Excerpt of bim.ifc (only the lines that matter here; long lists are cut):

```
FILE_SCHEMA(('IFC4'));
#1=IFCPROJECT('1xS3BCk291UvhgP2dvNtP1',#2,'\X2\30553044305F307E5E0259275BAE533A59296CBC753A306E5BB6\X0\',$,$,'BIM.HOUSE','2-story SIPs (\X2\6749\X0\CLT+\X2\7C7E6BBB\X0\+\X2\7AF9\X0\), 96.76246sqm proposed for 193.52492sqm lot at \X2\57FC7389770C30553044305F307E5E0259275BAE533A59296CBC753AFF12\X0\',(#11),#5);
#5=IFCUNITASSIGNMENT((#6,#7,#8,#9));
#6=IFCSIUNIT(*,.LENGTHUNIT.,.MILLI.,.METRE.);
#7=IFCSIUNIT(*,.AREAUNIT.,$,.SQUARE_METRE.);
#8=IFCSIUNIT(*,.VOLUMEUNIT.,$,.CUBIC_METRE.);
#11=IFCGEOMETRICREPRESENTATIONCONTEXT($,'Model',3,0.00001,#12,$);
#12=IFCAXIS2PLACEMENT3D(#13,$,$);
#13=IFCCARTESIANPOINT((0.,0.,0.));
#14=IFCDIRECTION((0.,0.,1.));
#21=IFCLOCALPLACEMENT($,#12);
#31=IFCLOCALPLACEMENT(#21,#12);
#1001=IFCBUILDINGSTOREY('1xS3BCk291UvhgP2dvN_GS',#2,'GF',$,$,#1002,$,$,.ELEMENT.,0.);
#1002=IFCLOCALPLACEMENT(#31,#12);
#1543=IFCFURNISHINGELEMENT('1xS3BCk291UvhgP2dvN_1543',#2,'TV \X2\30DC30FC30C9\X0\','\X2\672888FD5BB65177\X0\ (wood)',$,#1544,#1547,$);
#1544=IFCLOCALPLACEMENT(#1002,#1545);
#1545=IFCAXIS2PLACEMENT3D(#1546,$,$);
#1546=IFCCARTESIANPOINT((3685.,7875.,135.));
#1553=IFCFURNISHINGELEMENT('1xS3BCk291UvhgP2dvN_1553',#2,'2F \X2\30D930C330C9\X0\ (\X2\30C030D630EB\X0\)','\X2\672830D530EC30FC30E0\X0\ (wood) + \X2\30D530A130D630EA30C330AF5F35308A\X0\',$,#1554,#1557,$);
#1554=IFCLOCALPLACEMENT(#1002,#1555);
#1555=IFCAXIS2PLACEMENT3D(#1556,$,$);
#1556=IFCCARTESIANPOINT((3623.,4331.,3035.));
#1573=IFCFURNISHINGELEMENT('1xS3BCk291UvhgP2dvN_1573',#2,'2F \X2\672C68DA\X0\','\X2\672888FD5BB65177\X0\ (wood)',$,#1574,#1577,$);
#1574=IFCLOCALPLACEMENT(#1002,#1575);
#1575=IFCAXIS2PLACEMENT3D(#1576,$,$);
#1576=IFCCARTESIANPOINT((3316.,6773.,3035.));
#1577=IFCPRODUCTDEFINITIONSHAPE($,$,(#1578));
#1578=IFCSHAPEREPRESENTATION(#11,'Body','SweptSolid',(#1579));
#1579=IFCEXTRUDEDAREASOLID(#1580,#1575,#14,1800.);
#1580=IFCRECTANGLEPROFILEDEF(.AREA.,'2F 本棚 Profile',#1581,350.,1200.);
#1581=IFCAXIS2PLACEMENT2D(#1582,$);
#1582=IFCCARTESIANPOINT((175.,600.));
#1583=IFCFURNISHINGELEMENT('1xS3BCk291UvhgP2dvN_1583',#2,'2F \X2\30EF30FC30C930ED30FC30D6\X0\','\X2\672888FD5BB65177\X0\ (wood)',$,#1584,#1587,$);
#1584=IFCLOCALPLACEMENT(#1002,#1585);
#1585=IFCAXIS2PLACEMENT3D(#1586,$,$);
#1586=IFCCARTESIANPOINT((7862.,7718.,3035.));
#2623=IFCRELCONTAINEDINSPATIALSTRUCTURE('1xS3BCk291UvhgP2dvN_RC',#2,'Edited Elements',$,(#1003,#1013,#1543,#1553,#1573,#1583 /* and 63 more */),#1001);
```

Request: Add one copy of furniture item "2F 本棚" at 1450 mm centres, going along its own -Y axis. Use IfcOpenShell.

```python
import ifcopenshell
import ifcopenshell.api.geometry
import ifcopenshell.api.root
import ifcopenshell.util.element
import ifcopenshell.util.placement

model = ifcopenshell.open("bim.ifc")


def reuse_history(source, copy):
    """copy_class also copies each property set's owner history, people and application; keep the originals."""
    for rel in copy.IsDefinedBy:
        if rel.is_a("IfcRelDefinesByProperties") and (history := rel.RelatingPropertyDefinition.OwnerHistory):
            rel.RelatingPropertyDefinition.OwnerHistory = source.OwnerHistory
            ifcopenshell.util.element.remove_deep2(model, history)


source = model.by_guid("1xS3BCk291UvhgP2dvN_1573")
base = ifcopenshell.util.placement.get_local_placement(source.ObjectPlacement)
step = -base[:3, 1] * 1450.0

for i in range(1, 2):
    copy = ifcopenshell.api.root.copy_class(model, product=source)
    copy.Representation = ifcopenshell.util.element.copy_deep(
        model, source.Representation, exclude=["IfcGeometricRepresentationContext", "IfcRepresentationMap"]
    )
    reuse_history(source, copy)
    matrix = base.copy()
    matrix[:3, 3] += i * step
    print("added at", matrix[:3, 3].round(3) + 0.0)
    ifcopenshell.api.geometry.edit_object_placement(model, product=copy, matrix=matrix, is_si=False)

model.write("bim-out.ifc")
```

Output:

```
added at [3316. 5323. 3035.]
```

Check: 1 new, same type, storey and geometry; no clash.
